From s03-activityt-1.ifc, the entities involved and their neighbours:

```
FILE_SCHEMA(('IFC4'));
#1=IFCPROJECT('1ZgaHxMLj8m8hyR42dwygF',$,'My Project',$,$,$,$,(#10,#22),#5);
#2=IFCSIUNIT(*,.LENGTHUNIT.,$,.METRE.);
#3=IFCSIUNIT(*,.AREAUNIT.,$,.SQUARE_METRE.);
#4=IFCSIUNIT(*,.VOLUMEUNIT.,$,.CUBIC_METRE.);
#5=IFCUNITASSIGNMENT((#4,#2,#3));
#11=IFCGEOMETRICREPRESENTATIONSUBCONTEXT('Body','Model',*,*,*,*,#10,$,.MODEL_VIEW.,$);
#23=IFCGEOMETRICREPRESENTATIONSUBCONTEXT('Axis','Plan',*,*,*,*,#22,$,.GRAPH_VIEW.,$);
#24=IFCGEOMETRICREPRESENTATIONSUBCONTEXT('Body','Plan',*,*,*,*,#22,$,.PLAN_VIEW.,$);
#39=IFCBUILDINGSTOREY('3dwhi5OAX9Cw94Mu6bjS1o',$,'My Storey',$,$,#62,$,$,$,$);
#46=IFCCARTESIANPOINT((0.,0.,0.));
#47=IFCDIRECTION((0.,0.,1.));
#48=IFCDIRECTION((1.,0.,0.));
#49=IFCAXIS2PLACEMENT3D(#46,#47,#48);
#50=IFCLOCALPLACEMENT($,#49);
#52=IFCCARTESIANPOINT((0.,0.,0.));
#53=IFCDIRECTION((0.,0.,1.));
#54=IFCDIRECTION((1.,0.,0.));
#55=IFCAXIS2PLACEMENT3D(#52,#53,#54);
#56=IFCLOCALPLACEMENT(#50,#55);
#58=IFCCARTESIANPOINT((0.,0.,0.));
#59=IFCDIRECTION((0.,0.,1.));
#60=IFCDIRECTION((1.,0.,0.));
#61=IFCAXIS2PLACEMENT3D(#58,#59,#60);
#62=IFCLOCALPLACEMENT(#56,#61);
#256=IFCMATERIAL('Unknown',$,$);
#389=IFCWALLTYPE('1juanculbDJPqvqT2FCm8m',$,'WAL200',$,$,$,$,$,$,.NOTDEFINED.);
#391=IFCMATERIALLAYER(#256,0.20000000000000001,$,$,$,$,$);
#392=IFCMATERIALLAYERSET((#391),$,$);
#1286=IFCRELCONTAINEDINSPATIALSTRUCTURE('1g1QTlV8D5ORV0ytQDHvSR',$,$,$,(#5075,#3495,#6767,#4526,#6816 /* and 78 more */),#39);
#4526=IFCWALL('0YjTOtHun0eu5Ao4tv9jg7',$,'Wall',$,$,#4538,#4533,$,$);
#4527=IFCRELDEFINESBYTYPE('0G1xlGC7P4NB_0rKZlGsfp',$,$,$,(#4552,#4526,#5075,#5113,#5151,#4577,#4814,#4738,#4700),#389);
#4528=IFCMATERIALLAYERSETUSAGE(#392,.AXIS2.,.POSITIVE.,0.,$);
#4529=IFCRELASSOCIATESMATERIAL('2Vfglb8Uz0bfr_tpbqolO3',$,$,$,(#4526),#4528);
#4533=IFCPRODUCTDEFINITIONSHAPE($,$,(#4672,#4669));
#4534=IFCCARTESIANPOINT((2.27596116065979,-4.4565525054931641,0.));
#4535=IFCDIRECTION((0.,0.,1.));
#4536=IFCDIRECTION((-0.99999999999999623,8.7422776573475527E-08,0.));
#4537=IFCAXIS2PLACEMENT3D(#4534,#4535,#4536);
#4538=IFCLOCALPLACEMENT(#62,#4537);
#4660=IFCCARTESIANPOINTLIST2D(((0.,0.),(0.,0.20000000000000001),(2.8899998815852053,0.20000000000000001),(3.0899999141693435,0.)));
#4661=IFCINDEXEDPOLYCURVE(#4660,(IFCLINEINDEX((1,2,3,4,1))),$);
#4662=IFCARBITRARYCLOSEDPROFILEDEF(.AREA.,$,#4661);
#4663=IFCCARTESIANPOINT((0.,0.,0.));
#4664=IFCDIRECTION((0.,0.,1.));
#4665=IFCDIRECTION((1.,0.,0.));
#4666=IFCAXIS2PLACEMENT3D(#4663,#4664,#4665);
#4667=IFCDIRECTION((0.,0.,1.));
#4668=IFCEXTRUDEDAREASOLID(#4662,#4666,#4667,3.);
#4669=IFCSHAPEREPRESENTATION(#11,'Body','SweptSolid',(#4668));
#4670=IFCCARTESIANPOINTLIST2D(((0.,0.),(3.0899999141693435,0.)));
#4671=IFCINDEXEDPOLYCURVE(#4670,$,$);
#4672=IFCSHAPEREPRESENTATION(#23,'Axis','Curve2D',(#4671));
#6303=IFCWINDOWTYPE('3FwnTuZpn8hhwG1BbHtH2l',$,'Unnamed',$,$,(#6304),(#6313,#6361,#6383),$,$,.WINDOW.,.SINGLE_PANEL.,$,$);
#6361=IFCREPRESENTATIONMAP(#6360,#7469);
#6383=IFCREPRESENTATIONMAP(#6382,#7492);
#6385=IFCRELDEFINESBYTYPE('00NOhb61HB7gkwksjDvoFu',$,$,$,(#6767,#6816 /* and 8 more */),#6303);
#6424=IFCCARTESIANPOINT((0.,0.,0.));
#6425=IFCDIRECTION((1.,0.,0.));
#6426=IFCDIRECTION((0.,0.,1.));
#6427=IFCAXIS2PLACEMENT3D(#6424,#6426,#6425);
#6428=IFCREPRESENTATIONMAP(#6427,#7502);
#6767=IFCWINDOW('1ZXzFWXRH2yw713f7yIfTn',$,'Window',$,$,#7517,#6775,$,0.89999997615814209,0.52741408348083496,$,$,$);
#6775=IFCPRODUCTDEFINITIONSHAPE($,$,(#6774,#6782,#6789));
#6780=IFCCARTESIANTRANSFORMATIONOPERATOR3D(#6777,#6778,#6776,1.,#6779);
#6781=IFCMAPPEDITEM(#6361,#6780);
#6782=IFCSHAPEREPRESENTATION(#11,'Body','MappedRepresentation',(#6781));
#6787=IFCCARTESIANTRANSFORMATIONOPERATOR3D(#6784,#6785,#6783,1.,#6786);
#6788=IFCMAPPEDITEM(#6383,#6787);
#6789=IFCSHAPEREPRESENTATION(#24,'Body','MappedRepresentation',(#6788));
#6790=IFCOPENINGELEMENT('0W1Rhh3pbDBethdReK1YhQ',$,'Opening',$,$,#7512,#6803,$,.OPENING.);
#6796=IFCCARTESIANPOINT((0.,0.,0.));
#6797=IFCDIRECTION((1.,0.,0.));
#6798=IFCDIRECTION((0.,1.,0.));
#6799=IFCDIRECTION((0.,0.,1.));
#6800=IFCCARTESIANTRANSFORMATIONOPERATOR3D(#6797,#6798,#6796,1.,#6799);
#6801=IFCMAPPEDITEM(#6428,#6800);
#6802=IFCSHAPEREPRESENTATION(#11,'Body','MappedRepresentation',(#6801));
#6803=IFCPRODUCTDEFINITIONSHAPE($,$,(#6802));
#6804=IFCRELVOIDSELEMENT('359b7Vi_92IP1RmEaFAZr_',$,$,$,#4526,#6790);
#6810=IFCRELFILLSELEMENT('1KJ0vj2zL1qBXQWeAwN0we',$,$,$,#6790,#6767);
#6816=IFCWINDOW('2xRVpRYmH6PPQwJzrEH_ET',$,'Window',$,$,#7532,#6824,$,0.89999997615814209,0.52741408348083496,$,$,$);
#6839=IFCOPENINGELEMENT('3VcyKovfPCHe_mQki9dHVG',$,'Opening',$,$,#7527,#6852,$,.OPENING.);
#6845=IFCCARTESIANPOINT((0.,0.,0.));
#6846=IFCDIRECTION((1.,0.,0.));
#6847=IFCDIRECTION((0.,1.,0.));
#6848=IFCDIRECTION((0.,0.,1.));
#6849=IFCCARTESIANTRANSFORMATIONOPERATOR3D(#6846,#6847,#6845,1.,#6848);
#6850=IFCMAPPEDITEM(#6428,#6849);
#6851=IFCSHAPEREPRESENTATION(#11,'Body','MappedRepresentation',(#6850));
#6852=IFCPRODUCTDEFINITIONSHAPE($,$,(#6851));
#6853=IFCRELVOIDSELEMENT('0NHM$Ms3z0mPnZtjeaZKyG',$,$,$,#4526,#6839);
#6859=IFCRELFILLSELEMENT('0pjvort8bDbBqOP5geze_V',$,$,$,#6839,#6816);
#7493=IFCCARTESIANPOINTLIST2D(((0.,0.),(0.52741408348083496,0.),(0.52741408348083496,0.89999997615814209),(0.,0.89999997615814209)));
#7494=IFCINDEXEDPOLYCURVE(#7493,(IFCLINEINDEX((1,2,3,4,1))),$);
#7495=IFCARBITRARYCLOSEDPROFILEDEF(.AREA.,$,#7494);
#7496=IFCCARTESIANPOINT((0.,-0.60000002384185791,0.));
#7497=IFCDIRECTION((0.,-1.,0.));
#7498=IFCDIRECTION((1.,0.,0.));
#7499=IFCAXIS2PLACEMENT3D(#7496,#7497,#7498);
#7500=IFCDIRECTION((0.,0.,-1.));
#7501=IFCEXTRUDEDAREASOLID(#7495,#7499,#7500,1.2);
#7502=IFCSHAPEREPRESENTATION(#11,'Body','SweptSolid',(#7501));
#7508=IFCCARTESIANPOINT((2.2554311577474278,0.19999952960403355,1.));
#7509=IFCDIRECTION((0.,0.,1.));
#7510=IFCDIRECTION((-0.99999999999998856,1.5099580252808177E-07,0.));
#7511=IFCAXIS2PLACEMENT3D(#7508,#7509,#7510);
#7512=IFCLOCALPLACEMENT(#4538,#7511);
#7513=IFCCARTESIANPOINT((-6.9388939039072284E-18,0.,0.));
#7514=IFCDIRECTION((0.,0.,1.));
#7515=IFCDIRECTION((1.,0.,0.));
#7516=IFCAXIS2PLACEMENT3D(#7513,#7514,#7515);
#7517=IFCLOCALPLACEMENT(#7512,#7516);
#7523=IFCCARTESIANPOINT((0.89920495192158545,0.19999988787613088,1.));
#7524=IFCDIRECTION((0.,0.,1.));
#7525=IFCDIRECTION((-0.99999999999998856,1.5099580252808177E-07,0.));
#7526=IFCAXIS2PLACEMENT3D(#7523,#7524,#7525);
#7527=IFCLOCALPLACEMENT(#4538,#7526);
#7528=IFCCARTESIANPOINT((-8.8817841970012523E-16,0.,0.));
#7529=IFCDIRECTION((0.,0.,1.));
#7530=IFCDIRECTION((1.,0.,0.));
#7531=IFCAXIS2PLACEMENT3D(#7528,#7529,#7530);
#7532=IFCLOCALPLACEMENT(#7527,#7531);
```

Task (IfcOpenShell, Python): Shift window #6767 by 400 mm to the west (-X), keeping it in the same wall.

```python
import ifcopenshell
import ifcopenshell.api.geometry
import ifcopenshell.util.placement
import ifcopenshell.util.unit

model = ifcopenshell.open("s03-activityt-1.ifc")
unit_scale = ifcopenshell.util.unit.calculate_unit_scale(model)

window = model.by_id(6767)
opening = window.FillsVoids[0].RelatingOpeningElement
wall = opening.VoidsElements[0].RelatingBuildingElement

wall_matrix = ifcopenshell.util.placement.get_local_placement(wall.ObjectPlacement)
shift = wall_matrix[:3, 0] * 0.4 / unit_scale
before = ifcopenshell.util.placement.get_local_placement(window.ObjectPlacement)[:3, 3].copy()

# The window is placed relative to its opening, so it follows when the opening moves.
matrix = ifcopenshell.util.placement.get_local_placement(opening.ObjectPlacement)
matrix[:3, 3] += shift
ifcopenshell.api.geometry.edit_object_placement(
    model, product=opening, matrix=matrix, is_si=False, should_transform_children=True
)

after = ifcopenshell.util.placement.get_local_placement(window.ObjectPlacement)[:3, 3]
print("window moved by", (after - before).round(3) + 0.0)

model.write("s03-activityt-1_v2.ifc")
```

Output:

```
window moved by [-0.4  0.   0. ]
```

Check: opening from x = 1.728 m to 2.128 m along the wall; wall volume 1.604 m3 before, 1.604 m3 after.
